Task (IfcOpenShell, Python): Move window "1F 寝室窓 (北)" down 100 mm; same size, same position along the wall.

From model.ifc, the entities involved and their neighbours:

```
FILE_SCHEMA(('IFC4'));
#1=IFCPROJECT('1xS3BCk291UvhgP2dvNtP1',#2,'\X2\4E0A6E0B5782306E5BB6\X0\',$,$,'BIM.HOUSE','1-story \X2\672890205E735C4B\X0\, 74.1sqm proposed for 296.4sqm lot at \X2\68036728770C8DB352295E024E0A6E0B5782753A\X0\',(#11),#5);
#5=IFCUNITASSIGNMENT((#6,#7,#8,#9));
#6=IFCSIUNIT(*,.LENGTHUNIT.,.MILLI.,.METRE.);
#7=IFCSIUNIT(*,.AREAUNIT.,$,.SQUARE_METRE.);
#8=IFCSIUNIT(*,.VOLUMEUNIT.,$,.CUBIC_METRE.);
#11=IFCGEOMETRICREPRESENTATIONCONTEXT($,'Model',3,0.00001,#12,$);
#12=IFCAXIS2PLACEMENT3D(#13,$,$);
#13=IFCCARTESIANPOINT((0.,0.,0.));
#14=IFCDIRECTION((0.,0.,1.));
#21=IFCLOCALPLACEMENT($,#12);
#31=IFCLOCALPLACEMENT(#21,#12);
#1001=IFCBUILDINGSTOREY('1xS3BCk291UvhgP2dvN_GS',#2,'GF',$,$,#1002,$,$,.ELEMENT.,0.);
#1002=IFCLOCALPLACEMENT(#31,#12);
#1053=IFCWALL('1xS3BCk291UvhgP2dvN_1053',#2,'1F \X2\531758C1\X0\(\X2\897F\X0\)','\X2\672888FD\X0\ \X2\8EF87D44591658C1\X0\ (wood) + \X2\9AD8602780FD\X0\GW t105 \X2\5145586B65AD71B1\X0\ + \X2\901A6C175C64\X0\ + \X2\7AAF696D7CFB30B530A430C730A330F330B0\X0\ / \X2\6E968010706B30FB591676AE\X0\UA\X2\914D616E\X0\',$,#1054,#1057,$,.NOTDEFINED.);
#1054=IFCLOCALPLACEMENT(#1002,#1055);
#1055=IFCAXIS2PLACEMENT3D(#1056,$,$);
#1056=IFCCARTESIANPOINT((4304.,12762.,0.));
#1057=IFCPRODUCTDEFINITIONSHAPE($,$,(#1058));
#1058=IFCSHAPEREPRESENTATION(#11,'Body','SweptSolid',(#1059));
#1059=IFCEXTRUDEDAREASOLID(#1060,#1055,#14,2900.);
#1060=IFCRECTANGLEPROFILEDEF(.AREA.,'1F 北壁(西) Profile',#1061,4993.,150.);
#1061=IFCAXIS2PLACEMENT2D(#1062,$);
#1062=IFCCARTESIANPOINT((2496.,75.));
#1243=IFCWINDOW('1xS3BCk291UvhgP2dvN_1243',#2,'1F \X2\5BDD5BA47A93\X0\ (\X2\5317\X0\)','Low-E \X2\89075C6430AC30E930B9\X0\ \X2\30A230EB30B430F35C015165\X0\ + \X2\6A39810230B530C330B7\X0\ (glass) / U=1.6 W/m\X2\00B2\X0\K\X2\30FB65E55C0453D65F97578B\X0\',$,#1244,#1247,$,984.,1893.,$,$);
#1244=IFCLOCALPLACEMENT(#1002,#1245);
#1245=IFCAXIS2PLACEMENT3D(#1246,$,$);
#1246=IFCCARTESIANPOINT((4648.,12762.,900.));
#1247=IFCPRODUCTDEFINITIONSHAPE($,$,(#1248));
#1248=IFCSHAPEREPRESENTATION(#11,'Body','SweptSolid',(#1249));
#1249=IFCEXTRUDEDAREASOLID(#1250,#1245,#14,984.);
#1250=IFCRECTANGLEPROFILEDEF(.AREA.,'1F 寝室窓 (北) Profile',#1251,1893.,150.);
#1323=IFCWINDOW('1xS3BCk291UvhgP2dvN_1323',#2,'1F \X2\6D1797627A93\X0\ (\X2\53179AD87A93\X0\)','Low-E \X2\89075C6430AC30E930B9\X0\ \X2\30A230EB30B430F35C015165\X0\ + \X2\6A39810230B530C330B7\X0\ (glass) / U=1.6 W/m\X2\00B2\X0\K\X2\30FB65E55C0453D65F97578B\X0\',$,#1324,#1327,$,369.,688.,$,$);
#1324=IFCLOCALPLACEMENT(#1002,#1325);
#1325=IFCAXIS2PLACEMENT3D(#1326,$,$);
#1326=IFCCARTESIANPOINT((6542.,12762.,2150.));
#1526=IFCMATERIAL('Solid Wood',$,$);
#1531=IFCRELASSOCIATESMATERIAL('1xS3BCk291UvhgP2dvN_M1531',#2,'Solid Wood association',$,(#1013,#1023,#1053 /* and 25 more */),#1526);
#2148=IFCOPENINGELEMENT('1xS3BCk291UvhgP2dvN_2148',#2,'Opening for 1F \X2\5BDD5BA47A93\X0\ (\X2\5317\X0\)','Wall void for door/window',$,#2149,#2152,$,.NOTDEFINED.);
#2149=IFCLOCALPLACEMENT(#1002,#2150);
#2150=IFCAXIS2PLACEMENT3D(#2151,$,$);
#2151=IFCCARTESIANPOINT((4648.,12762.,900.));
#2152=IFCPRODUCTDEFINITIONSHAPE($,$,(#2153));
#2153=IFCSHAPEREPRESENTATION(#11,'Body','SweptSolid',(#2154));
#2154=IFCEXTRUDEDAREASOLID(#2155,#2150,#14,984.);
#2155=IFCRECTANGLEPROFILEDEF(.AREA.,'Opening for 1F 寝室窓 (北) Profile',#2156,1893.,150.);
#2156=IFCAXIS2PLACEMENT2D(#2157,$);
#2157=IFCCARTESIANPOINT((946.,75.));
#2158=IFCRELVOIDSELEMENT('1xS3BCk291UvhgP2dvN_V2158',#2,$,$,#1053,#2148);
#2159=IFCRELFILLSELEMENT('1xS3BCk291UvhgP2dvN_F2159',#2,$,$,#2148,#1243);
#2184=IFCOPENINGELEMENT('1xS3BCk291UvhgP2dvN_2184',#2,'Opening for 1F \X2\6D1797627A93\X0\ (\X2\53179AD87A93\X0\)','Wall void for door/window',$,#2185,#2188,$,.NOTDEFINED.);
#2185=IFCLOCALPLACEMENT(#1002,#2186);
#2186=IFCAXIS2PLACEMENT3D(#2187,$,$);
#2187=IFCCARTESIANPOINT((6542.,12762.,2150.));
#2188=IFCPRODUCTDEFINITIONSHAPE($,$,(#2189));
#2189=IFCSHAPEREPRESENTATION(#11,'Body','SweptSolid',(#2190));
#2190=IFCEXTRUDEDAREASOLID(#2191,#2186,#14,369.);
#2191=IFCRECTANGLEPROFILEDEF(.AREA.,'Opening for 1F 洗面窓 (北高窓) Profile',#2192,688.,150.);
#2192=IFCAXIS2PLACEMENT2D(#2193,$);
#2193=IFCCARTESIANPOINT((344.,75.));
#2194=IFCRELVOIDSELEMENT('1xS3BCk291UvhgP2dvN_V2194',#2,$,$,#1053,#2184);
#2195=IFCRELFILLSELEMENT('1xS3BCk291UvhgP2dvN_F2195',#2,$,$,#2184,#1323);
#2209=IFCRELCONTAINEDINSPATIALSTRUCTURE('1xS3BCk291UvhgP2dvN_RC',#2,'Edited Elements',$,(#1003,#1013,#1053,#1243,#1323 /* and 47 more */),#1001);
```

```python
import numpy as np
import ifcopenshell
import ifcopenshell.api.geometry
import ifcopenshell.util.placement
import ifcopenshell.util.unit

model = ifcopenshell.open("model.ifc")
unit_scale = ifcopenshell.util.unit.calculate_unit_scale(model)

window = model.by_guid("1xS3BCk291UvhgP2dvN_1243")
opening = window.FillsVoids[0].RelatingOpeningElement
dz = -100.0

shift = np.array([0.0, 0.0, dz])
# The window is not placed relative to its opening, so move both.
for product in (opening, window):
    matrix = ifcopenshell.util.placement.get_local_placement(product.ObjectPlacement)
    matrix[:3, 3] += shift
    ifcopenshell.api.geometry.edit_object_placement(model, product=product, matrix=matrix, is_si=False)

print(f"moved by {dz * unit_scale:+.3f} m")

model.write("model_v2.ifc")
```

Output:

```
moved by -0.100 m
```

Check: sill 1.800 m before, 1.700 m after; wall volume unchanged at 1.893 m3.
